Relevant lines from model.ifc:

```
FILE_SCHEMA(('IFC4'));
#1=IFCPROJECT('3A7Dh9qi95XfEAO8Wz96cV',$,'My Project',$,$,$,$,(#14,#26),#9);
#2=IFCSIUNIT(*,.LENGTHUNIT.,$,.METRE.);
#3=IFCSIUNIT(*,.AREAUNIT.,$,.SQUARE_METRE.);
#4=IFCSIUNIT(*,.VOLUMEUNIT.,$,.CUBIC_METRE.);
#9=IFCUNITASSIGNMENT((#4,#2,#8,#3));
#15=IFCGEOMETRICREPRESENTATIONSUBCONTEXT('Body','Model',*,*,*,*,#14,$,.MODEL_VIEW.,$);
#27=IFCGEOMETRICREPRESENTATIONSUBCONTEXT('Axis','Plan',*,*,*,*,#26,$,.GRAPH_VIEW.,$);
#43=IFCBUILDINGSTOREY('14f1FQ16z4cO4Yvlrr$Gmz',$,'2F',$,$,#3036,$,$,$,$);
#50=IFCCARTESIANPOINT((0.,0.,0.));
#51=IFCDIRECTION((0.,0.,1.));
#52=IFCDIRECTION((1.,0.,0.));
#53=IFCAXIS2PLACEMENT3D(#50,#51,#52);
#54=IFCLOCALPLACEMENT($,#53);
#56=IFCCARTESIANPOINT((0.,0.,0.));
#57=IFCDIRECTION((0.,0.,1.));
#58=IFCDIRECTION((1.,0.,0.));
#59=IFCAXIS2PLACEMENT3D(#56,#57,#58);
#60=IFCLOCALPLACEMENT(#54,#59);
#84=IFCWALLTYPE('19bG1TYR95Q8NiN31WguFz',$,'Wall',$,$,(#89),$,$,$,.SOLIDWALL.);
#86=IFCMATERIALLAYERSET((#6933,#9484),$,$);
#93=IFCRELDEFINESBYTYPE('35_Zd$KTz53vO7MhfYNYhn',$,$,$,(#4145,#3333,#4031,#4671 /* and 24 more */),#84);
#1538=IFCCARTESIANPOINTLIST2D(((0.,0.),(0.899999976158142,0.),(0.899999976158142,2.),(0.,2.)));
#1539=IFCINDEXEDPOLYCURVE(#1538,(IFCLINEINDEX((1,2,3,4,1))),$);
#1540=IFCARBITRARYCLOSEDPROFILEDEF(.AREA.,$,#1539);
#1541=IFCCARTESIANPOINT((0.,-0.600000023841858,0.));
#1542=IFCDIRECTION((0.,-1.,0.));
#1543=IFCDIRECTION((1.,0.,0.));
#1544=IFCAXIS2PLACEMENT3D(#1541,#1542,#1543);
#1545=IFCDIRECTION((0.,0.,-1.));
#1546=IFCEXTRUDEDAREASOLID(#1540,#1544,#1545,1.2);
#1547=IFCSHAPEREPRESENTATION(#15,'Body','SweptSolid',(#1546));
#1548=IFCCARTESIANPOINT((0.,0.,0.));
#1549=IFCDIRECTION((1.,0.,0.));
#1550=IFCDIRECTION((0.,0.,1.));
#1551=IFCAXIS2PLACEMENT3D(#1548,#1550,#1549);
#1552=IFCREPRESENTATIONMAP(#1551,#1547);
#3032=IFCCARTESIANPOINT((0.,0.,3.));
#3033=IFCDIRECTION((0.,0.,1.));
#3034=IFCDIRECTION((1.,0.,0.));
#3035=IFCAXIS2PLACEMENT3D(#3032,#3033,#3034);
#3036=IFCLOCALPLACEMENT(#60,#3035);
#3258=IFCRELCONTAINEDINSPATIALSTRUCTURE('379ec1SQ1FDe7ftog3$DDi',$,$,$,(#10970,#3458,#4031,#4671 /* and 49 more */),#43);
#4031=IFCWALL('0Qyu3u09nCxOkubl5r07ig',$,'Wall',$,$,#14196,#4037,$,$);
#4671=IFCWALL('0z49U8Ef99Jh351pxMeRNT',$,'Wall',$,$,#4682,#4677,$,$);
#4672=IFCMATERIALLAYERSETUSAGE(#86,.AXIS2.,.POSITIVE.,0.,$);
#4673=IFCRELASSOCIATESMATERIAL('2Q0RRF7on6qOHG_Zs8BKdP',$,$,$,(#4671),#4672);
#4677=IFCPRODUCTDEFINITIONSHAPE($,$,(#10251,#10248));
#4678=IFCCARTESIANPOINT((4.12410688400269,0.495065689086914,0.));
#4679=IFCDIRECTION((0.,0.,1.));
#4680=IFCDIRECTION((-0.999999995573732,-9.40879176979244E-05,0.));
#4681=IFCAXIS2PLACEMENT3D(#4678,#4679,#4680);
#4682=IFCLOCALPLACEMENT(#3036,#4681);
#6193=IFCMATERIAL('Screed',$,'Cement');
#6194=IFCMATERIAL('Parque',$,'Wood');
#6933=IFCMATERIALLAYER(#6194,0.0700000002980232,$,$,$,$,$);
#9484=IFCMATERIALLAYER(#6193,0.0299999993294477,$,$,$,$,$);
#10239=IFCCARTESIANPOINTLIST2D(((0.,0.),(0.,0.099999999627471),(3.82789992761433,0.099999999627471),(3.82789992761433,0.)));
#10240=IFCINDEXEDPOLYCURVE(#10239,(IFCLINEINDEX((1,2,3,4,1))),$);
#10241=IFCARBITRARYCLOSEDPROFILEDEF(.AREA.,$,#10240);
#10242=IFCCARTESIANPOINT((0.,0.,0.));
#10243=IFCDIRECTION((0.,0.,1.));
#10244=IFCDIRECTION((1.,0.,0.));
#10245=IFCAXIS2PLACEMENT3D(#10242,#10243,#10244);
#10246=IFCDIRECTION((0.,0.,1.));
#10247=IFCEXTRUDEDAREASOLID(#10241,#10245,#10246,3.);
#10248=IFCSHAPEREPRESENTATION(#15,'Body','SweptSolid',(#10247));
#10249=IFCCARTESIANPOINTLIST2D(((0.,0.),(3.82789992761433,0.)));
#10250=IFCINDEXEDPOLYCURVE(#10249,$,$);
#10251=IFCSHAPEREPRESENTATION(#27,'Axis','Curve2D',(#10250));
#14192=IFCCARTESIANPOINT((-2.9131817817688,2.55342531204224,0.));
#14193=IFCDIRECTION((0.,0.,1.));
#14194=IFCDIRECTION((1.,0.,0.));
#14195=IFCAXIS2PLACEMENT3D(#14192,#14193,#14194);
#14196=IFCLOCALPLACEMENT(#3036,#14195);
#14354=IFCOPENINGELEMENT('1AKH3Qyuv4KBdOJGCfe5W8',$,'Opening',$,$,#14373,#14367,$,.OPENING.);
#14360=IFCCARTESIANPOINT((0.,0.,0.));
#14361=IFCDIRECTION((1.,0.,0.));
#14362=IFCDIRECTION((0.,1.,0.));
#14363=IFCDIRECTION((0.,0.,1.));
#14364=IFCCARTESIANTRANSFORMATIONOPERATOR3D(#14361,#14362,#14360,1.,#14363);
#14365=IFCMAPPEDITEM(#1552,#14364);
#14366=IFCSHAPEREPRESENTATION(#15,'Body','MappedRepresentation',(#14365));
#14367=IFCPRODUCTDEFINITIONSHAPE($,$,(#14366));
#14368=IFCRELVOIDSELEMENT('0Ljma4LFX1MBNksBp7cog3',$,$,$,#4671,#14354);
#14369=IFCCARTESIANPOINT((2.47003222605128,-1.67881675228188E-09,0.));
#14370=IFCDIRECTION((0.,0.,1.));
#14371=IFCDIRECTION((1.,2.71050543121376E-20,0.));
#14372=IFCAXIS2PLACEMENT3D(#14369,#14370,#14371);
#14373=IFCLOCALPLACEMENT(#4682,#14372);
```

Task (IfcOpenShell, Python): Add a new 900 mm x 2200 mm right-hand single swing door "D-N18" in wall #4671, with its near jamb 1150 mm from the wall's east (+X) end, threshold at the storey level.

```python
import numpy as np
import ifcopenshell
import ifcopenshell.api.feature
import ifcopenshell.api.geometry
import ifcopenshell.api.root
import ifcopenshell.api.spatial
import ifcopenshell.geom
import ifcopenshell.util.element
import ifcopenshell.util.placement
import ifcopenshell.util.representation
import ifcopenshell.util.shape
import ifcopenshell.util.unit

model = ifcopenshell.open("model.ifc")
unit_scale = ifcopenshell.util.unit.calculate_unit_scale(model)
settings = ifcopenshell.geom.settings()


def volume(element):
    """Net volume in cubic metres, openings subtracted."""
    shape = ifcopenshell.geom.create_shape(settings, element)
    return ifcopenshell.util.shape.get_volume(shape.geometry)


wall = model.by_guid("0z49U8Ef99Jh351pxMeRNT")
storey = ifcopenshell.util.element.get_container(wall, ifc_class="IfcBuildingStorey")
context = ifcopenshell.util.representation.get_context(model, "Model", "Body", "MODEL_VIEW")
before = volume(wall)

width, height, from_end, sill = 0.9, 2.2, 1.15, 0.0  # metres

# The wall runs along its own X axis, and the end named is its -X end.
wall_shape = ifcopenshell.geom.create_shape(settings, wall)
x, y, z = ifcopenshell.util.shape.get_vertices(wall_shape.geometry).T
start = x.min() + from_end
face, thickness = float(y.min()), float(y.max() - y.min())
wall_matrix = ifcopenshell.util.placement.get_local_placement(wall.ObjectPlacement)
level = ifcopenshell.util.placement.get_local_placement(storey.ObjectPlacement)[2, 3]


def in_wall(x, y):
    """Placement at x, y metres in the wall's axes, at sill height."""
    matrix = wall_matrix.copy()
    matrix[:, 3] = wall_matrix @ np.array([x / unit_scale, y / unit_scale, 0.0, 1.0])
    matrix[2, 3] = level + sill / unit_scale
    return matrix


# Opening: a box that overshoots both wall faces by 50 mm.
opening = ifcopenshell.api.root.create_entity(model, ifc_class="IfcOpeningElement", predefined_type="OPENING")
box = ifcopenshell.api.geometry.add_wall_representation(
    model, context=context, length=width, height=height, thickness=thickness + 0.1
)
ifcopenshell.api.geometry.assign_representation(model, product=opening, representation=box)
ifcopenshell.api.geometry.edit_object_placement(model, product=opening, matrix=in_wall(start, face - 0.05), is_si=False)
ifcopenshell.api.feature.add_feature(model, feature=opening, element=wall)

door = ifcopenshell.api.root.create_entity(model, ifc_class="IfcDoor", name="D-N18", predefined_type="DOOR")
door.OverallWidth, door.OverallHeight = width / unit_scale, height / unit_scale
door.OperationType = "SINGLE_SWING_RIGHT"
body = ifcopenshell.api.geometry.add_door_representation(
    model,
    context=context,
    overall_width=door.OverallWidth,
    overall_height=door.OverallHeight,
    operation_type="SINGLE_SWING_RIGHT",
    lining_properties={"LiningDepth": thickness / unit_scale, "ThresholdDepth": thickness / unit_scale},
)
ifcopenshell.api.geometry.assign_representation(model, product=door, representation=body)
ifcopenshell.api.spatial.assign_container(model, products=[door], relating_structure=storey)
ifcopenshell.api.feature.add_filling(model, opening=opening, element=door)

# The lining spans the wall, so the door starts at the wall face.
ifcopenshell.api.geometry.edit_object_placement(model, product=door, matrix=in_wall(start, face), is_si=False)

after = volume(wall)

print(f"wall volume {before:.3f} -> {after:.3f} m3")

model.write("model_updated.ifc")
```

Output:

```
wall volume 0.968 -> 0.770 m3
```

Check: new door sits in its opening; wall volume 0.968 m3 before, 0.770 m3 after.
